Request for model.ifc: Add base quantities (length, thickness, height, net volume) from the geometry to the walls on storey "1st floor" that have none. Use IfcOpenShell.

First a look at what the model holds.

```python
import ifcopenshell
import ifcopenshell.util.element
import ifcopenshell.util.unit

model = ifcopenshell.open("model.ifc")
print(model.schema)
for unit_type in ("LENGTHUNIT", "AREAUNIT", "VOLUMEUNIT"):
    print(unit_type, ifcopenshell.util.unit.calculate_unit_scale(model, unit_type))
storey = next(s for s in model.by_type("IfcBuildingStorey") if s.Name == "1st floor")
walls = [e for e in ifcopenshell.util.element.get_decomposition(storey) if e.is_a("IfcWall")]
for e in sorted(walls, key=lambda e: e.id()):
    print(e.id(), e.is_a(), e.Name, list(ifcopenshell.util.element.get_psets(e, qtos_only=True)), sep=" | ")
```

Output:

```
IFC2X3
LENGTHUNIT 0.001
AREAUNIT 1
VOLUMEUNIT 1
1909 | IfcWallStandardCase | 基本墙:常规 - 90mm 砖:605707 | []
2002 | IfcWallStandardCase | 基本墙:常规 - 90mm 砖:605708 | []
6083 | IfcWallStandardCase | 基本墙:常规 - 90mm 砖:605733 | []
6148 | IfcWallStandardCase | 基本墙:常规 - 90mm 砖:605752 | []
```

```python
import ifcopenshell
import ifcopenshell.api.pset
import ifcopenshell.geom
import ifcopenshell.util.element
import ifcopenshell.util.shape
import ifcopenshell.util.unit

model = ifcopenshell.open("model.ifc")
unit_scale = ifcopenshell.util.unit.calculate_unit_scale(model)
volume_scale = ifcopenshell.util.unit.calculate_unit_scale(model, "VOLUMEUNIT")
settings = ifcopenshell.geom.settings()

storey = next(s for s in model.by_type("IfcBuildingStorey") if s.Name == "1st floor")
walls = [e for e in ifcopenshell.util.element.get_decomposition(storey) if e.is_a("IfcWall")]

for e in sorted(walls, key=lambda e: e.id()):
    if ifcopenshell.util.element.get_psets(e, qtos_only=True, should_inherit=False):
        continue
    # Geometry comes back in metres, in the element's own axes.
    shape = ifcopenshell.geom.create_shape(settings, e)
    values = {
        "Length": ifcopenshell.util.shape.get_x(shape.geometry) / unit_scale,
        "Width": ifcopenshell.util.shape.get_y(shape.geometry) / unit_scale,
        "Height": ifcopenshell.util.shape.get_z(shape.geometry) / unit_scale,
        "NetVolume": ifcopenshell.util.shape.get_volume(shape.geometry) / volume_scale,
    }
    qto = ifcopenshell.api.pset.add_qto(model, product=e, name="BaseQuantities")
    ifcopenshell.api.pset.edit_qto(model, qto=qto, properties=values)
    print(e.id(), {k: round(v, 3) for k, v in values.items()})

model.write("model_v2.ifc")
```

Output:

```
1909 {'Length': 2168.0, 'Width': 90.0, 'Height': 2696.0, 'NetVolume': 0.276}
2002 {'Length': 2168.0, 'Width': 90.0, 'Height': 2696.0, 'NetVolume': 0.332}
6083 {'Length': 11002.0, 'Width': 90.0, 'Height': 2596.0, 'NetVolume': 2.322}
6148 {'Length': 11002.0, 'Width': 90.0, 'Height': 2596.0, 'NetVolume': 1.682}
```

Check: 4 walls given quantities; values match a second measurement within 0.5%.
